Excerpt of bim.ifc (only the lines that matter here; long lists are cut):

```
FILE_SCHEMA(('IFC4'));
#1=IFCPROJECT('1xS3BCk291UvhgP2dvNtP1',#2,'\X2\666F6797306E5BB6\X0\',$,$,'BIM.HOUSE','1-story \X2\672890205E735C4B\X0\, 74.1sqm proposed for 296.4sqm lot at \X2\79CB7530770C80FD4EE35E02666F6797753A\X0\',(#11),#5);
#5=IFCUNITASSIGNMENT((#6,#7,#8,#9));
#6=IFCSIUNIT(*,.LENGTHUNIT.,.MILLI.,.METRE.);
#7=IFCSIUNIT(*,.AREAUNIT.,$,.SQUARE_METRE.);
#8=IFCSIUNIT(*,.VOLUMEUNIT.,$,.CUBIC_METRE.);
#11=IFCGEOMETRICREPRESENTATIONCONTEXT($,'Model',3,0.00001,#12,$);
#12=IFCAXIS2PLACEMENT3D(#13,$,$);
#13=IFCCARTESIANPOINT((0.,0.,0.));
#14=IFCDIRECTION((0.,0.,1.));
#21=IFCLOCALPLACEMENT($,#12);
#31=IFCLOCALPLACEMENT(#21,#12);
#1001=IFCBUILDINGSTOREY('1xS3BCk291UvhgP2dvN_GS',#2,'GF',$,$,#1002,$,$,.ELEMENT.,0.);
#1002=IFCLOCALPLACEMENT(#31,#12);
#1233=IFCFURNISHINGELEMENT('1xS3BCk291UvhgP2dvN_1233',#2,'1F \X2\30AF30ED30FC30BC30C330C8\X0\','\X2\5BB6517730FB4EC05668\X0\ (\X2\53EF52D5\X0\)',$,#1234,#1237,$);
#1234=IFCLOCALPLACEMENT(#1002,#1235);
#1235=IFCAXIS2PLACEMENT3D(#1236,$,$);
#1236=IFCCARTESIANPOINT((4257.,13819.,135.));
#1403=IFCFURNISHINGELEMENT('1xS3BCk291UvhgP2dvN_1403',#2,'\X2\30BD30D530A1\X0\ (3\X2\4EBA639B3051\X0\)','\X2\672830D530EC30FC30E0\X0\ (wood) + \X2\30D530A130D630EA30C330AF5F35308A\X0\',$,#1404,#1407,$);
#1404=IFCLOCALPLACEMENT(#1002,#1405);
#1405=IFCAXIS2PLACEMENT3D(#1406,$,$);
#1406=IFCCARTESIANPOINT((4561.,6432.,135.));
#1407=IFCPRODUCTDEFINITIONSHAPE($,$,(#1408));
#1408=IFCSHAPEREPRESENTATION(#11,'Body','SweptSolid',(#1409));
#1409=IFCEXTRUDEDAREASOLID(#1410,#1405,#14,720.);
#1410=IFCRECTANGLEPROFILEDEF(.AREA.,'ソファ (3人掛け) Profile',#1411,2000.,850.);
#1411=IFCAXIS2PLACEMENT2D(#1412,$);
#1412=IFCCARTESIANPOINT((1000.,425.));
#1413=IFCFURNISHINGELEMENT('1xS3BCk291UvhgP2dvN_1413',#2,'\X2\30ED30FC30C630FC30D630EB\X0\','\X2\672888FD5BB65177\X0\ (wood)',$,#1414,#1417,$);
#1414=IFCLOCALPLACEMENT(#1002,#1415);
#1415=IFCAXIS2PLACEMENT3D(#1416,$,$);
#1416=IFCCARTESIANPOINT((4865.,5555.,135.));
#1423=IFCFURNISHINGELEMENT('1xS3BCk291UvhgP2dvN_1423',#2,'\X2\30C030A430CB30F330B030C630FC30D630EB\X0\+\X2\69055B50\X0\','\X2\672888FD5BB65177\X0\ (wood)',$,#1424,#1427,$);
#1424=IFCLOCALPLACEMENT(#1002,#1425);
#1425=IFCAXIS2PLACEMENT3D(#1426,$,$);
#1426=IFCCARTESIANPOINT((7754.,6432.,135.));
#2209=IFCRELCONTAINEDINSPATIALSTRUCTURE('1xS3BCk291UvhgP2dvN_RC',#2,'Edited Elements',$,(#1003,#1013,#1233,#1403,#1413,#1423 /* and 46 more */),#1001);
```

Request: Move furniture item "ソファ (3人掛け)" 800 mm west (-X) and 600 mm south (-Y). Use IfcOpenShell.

```python
import ifcopenshell
import ifcopenshell.api.geometry
import ifcopenshell.util.placement

model = ifcopenshell.open("bim.ifc")

item = model.by_id(1403)
matrix = ifcopenshell.util.placement.get_local_placement(item.ObjectPlacement)
matrix[0, 3] -= 800.0
matrix[1, 3] -= 600.0
ifcopenshell.api.geometry.edit_object_placement(model, product=item, matrix=matrix, is_si=False)

print(ifcopenshell.util.placement.get_local_placement(item.ObjectPlacement).round(3) + 0.0)

model.write("bim-out.ifc")
```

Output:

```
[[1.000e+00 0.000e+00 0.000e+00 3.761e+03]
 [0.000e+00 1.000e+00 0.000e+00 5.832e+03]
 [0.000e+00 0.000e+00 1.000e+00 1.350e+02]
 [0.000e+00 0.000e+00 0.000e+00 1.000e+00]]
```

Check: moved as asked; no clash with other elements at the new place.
